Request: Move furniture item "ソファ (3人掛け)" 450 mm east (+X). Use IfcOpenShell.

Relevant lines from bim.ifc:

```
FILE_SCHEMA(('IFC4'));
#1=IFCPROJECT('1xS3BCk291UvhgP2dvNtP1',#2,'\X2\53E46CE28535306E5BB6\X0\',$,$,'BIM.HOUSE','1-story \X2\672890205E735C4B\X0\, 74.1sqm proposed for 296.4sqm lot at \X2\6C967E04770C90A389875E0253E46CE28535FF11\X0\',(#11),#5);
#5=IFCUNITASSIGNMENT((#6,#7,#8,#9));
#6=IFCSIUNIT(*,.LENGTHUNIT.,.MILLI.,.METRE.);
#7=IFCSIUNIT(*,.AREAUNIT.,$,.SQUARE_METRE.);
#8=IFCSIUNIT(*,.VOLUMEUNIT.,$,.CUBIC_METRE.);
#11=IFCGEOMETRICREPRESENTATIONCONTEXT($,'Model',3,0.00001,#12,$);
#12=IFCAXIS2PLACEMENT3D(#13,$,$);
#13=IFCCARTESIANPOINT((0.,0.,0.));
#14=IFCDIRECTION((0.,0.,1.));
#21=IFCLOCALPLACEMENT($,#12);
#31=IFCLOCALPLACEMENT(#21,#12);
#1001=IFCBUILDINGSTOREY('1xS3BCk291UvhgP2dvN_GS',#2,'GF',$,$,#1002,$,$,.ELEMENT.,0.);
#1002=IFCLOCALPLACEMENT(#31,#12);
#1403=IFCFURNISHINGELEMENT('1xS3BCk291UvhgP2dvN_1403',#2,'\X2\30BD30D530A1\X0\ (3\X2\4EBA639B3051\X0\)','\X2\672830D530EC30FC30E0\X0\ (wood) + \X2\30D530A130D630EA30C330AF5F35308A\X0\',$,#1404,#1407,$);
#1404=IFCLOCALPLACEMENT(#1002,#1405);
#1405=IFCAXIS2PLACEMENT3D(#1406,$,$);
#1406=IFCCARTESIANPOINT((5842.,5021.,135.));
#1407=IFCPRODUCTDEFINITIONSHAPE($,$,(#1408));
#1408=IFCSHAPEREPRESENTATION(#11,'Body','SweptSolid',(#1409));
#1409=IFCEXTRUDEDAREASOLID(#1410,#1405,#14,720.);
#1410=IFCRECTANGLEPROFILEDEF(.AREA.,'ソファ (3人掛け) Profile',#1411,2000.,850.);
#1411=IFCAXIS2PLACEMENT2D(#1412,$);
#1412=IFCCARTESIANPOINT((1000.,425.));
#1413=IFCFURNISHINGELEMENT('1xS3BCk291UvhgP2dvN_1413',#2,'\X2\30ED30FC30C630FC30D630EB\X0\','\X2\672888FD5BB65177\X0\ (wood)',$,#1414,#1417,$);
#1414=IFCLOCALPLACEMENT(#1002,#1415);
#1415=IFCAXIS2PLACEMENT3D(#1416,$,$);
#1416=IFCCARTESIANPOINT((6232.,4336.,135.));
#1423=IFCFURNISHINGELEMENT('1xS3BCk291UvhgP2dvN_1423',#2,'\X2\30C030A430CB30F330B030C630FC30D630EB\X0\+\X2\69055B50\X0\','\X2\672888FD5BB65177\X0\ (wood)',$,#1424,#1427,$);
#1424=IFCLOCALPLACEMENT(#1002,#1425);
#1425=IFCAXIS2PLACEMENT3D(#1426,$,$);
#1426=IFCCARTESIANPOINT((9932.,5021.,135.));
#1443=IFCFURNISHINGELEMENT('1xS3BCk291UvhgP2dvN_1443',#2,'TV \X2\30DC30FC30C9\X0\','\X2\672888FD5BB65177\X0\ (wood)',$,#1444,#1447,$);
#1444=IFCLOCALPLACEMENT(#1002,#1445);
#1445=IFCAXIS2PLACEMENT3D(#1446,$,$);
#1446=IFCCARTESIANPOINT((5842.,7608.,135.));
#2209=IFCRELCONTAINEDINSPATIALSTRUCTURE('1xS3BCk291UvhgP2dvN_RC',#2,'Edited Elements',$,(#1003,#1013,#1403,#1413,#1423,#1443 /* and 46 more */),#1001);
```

```python
import ifcopenshell
import ifcopenshell.api.geometry
import ifcopenshell.util.placement

model = ifcopenshell.open("bim.ifc")

item = model.by_guid("1xS3BCk291UvhgP2dvN_1403")
matrix = ifcopenshell.util.placement.get_local_placement(item.ObjectPlacement)
matrix[0, 3] += 450.0
ifcopenshell.api.geometry.edit_object_placement(model, product=item, matrix=matrix, is_si=False)

print(ifcopenshell.util.placement.get_local_placement(item.ObjectPlacement).round(3) + 0.0)

model.write("bim_v2.ifc")
```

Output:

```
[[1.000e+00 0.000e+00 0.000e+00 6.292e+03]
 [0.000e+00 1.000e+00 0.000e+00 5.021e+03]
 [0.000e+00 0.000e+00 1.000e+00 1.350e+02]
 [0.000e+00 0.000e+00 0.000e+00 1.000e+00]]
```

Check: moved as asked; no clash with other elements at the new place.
